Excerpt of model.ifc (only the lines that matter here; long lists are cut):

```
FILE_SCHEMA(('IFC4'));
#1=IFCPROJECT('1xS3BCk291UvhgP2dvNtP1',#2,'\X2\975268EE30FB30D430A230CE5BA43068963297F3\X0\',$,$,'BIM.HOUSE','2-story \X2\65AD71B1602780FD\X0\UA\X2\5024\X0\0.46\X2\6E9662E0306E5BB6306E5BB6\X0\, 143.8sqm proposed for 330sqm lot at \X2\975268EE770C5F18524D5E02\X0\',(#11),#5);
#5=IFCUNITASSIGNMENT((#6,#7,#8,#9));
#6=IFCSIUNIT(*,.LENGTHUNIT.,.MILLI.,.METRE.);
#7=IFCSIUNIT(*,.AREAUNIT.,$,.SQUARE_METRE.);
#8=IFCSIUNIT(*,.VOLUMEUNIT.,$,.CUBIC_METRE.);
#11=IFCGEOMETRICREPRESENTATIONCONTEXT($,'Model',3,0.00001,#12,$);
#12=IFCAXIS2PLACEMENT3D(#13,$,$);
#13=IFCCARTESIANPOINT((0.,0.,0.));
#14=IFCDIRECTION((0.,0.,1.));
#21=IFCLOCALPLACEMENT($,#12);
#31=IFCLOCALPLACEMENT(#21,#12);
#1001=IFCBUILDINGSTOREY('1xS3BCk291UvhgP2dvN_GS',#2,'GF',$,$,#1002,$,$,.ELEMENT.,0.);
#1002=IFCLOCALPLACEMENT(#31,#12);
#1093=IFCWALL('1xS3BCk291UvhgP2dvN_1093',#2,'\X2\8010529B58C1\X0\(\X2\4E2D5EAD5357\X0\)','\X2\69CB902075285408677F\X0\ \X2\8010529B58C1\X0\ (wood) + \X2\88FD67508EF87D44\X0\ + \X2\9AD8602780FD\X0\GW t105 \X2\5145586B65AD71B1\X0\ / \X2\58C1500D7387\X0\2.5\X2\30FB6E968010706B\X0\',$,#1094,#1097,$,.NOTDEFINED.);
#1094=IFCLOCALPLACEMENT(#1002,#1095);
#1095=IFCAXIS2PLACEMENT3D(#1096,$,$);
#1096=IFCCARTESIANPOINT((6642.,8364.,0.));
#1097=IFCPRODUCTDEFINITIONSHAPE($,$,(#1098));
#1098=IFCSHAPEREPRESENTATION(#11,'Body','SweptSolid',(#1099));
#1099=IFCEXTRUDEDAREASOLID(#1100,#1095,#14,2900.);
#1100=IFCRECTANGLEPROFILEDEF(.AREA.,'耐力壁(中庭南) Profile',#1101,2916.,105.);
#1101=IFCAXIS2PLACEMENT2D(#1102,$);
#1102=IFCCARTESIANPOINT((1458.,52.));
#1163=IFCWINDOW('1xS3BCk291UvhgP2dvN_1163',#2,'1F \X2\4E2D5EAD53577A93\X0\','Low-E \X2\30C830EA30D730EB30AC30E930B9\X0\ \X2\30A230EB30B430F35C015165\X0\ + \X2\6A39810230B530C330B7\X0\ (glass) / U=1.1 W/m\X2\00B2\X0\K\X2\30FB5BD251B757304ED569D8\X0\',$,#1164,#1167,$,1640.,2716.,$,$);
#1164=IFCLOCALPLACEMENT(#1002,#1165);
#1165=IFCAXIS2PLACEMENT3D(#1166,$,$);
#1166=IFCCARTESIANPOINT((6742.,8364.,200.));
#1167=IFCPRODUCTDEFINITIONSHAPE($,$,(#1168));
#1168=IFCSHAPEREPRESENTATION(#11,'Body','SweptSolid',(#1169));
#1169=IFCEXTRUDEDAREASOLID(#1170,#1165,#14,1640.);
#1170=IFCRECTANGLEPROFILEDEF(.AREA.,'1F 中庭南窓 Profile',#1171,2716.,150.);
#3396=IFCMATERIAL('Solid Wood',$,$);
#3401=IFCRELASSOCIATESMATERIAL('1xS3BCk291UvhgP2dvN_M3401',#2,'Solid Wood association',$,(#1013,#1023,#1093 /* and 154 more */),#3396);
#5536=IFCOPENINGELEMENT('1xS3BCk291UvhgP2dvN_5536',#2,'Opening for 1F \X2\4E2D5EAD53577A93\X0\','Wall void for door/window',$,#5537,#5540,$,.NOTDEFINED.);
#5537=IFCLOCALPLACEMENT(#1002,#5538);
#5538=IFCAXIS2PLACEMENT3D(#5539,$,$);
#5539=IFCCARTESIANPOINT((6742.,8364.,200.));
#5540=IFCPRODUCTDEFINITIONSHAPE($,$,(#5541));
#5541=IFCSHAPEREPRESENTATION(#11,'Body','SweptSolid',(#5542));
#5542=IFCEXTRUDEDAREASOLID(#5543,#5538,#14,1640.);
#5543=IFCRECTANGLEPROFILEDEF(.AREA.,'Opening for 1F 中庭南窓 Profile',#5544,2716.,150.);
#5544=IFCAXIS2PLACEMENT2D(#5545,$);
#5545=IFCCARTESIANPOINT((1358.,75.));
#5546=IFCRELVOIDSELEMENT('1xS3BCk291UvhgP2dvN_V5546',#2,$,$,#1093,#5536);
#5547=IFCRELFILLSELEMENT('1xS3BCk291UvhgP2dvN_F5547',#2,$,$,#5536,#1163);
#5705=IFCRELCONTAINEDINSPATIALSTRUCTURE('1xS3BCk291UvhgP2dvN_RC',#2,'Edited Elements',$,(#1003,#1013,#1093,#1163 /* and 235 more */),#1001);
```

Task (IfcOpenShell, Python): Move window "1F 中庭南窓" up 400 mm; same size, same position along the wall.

```python
import numpy as np
import ifcopenshell
import ifcopenshell.api.geometry
import ifcopenshell.util.placement
import ifcopenshell.util.unit

model = ifcopenshell.open("model.ifc")
unit_scale = ifcopenshell.util.unit.calculate_unit_scale(model)

window = model.by_guid("1xS3BCk291UvhgP2dvN_1163")
opening = window.FillsVoids[0].RelatingOpeningElement
dz = 0.4 / unit_scale

shift = np.array([0.0, 0.0, dz])
# The window is not placed relative to its opening, so move both.
for product in (opening, window):
    matrix = ifcopenshell.util.placement.get_local_placement(product.ObjectPlacement)
    matrix[:3, 3] += shift
    ifcopenshell.api.geometry.edit_object_placement(model, product=product, matrix=matrix, is_si=False)

print(f"moved by {dz * unit_scale:+.3f} m")

model.write("model_v2.ifc")
```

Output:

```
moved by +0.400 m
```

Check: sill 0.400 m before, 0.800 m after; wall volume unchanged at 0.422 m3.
